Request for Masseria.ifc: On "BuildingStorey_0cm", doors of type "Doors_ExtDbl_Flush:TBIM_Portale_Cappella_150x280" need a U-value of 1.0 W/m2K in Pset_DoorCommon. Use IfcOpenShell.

First a look at what the model holds.

```python
import ifcopenshell
import ifcopenshell.util.element

model = ifcopenshell.open("Masseria.ifc")
print(model.schema)
storey = next(s for s in model.by_type("IfcBuildingStorey") if s.Name == "BuildingStorey_0cm")
doors = [e for e in ifcopenshell.util.element.get_decomposition(storey) if e.is_a("IfcDoor")]
seen = {}
for e in doors:
    element_type = ifcopenshell.util.element.get_type(e)
    key = (element_type.Name if element_type != e and element_type else None, ifcopenshell.util.element.get_pset(e, "Pset_DoorCommon", "ThermalTransmittance"))
    seen[key] = seen.get(key, 0) + 1
for (name, value), count in sorted(seen.items(), key=str):
    print(count, "x", name, "|", value)
```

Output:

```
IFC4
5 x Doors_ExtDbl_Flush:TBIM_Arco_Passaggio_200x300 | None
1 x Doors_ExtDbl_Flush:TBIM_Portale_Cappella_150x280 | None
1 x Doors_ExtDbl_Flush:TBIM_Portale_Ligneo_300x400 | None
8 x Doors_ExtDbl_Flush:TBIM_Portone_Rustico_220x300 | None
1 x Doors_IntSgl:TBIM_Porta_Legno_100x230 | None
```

```python
import ifcopenshell
import ifcopenshell.api.pset
import ifcopenshell.util.element

model = ifcopenshell.open("Masseria.ifc")

storey = next(s for s in model.by_type("IfcBuildingStorey") if s.Name == "BuildingStorey_0cm")
doors = [e for e in ifcopenshell.util.element.get_decomposition(storey) if e.is_a("IfcDoor")]

count = 0
for e in doors:
    element_type = ifcopenshell.util.element.get_type(e)
    if element_type in (None, e) or element_type.Name != "Doors_ExtDbl_Flush:TBIM_Portale_Cappella_150x280":
        continue
    # add_pset returns the element's existing set when there is one.
    pset = ifcopenshell.api.pset.add_pset(model, product=e, name="Pset_DoorCommon")
    ifcopenshell.api.pset.edit_pset(model, pset=pset, properties={"ThermalTransmittance": 1.0})
    count += 1

print(count, "doors updated")

model.write("Masseria_rev.ifc")
```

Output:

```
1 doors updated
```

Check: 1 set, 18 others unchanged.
